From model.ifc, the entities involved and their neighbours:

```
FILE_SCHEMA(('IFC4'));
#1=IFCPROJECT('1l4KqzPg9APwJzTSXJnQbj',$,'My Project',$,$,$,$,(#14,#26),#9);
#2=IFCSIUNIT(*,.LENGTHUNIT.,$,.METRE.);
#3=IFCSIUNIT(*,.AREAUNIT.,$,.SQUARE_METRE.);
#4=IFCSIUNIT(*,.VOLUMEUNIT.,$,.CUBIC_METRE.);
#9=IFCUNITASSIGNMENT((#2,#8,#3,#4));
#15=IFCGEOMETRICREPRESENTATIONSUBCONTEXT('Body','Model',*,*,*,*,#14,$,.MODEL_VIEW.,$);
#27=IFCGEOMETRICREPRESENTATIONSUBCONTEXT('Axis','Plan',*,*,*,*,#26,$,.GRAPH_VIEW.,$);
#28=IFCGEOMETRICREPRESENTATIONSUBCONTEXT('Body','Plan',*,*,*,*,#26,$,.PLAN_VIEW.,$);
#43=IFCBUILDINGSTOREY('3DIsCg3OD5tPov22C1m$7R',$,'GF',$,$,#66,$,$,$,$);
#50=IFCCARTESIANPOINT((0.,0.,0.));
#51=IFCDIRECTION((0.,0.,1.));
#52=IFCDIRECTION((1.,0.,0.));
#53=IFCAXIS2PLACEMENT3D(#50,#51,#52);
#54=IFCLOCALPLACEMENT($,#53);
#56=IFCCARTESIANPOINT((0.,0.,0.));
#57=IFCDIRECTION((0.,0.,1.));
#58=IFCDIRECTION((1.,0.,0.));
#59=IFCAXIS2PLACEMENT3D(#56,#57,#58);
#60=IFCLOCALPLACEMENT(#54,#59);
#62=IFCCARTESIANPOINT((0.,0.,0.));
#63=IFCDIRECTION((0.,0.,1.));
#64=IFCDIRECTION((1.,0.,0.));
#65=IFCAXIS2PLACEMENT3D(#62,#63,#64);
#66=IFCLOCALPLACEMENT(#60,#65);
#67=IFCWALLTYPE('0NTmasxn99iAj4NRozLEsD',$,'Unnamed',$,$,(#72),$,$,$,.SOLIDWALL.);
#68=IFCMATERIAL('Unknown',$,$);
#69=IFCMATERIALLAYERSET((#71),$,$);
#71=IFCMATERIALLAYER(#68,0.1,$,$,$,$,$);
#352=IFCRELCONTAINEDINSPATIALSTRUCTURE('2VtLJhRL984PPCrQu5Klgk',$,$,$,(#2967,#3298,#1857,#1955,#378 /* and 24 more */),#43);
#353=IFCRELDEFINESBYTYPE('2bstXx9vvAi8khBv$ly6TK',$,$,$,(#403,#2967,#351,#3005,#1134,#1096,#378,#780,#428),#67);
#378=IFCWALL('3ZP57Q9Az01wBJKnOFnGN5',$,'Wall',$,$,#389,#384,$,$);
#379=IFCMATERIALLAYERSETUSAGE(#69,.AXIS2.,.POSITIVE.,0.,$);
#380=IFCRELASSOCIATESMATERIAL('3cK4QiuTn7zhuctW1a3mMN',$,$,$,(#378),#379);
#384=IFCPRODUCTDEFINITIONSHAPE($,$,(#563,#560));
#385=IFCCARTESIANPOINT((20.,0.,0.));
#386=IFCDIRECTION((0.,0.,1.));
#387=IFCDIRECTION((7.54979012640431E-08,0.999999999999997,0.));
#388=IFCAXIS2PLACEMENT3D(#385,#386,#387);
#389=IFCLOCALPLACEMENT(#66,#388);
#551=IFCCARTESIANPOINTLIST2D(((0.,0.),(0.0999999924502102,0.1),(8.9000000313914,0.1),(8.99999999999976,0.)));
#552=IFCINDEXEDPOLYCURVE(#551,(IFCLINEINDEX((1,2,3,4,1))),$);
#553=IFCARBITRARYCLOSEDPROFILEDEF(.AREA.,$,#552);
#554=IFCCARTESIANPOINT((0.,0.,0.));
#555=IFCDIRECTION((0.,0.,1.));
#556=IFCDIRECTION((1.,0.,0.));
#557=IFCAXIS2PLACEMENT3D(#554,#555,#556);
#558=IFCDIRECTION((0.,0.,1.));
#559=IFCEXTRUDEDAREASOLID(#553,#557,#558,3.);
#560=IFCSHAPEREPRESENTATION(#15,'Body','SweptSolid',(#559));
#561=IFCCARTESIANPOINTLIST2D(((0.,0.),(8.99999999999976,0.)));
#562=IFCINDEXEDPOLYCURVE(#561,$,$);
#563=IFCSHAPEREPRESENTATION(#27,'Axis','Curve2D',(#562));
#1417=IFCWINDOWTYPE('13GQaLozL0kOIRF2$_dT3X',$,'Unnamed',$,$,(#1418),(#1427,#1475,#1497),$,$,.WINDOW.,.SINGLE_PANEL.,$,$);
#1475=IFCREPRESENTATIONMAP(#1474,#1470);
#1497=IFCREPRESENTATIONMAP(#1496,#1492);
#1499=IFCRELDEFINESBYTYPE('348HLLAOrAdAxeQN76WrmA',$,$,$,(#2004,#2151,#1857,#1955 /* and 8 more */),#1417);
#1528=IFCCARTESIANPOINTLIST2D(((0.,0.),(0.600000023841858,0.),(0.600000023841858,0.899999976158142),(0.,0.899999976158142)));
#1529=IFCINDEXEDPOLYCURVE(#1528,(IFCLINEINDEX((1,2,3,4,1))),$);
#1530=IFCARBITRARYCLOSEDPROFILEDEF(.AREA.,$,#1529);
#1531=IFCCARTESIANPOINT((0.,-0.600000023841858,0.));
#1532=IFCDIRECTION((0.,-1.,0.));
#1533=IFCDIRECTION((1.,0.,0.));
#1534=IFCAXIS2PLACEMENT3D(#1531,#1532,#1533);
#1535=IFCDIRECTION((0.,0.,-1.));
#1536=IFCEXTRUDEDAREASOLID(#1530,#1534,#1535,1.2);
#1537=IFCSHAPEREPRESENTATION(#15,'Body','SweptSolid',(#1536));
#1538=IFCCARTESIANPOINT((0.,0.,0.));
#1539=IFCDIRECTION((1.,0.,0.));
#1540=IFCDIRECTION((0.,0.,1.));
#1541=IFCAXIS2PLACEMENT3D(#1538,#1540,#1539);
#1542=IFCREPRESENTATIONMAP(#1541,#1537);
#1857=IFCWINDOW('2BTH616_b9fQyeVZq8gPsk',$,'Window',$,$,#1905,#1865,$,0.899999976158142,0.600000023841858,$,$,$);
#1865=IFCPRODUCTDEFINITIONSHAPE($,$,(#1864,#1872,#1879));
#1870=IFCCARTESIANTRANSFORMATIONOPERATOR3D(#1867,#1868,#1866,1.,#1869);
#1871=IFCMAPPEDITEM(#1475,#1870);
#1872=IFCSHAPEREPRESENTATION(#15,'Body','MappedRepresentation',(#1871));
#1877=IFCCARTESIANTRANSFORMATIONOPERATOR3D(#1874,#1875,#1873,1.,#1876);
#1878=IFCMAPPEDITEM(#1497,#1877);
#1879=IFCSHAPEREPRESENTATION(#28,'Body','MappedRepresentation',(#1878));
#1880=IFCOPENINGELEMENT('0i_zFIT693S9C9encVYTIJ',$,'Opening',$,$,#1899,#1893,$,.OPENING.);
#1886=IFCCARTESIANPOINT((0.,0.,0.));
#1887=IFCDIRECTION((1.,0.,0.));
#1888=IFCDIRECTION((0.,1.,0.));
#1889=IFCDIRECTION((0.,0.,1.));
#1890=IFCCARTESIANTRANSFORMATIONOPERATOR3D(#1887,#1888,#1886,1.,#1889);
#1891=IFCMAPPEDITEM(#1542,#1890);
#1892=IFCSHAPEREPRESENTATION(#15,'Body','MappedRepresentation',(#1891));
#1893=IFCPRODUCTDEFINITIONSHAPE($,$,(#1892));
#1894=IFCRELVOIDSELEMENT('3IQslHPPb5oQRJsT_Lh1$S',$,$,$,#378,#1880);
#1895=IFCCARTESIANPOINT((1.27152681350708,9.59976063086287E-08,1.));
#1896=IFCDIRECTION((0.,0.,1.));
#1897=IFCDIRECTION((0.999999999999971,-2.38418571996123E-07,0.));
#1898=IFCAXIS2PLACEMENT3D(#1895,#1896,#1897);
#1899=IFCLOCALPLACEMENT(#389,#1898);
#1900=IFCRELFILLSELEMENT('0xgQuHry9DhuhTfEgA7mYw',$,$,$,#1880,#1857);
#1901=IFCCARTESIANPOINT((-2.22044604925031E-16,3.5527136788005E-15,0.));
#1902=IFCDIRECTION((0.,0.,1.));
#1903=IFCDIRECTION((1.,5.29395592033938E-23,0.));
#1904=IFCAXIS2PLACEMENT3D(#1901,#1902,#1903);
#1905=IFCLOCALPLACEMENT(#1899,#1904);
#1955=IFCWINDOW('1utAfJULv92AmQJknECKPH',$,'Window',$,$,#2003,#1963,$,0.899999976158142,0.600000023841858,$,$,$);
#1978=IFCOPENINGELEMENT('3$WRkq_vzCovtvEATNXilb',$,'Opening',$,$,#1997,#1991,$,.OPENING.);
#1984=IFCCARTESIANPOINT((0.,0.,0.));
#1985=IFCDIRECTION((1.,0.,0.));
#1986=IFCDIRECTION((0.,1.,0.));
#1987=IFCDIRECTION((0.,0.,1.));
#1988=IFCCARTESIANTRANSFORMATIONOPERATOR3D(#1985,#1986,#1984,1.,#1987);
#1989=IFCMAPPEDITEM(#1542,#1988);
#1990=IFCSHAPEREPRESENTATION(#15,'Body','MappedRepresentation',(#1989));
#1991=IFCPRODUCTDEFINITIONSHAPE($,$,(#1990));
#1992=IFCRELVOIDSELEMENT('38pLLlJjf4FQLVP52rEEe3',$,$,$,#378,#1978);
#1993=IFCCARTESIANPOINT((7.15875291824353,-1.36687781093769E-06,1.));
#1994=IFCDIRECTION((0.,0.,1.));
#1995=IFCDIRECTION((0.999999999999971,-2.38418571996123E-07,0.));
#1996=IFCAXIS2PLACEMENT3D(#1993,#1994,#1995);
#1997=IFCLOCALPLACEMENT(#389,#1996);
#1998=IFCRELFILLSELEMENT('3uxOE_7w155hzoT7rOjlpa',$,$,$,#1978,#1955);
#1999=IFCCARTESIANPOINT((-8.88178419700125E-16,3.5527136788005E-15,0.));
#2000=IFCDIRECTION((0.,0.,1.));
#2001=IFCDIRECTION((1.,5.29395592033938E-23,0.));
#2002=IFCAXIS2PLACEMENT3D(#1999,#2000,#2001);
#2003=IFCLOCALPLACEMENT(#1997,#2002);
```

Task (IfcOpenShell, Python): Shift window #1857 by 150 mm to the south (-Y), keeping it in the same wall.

```python
import ifcopenshell
import ifcopenshell.api.geometry
import ifcopenshell.util.placement
import ifcopenshell.util.unit

model = ifcopenshell.open("model.ifc")
unit_scale = ifcopenshell.util.unit.calculate_unit_scale(model)

window = model.by_guid("2BTH616_b9fQyeVZq8gPsk")
opening = window.FillsVoids[0].RelatingOpeningElement
wall = opening.VoidsElements[0].RelatingBuildingElement

wall_matrix = ifcopenshell.util.placement.get_local_placement(wall.ObjectPlacement)
shift = wall_matrix[:3, 0] * -0.15 / unit_scale
before = ifcopenshell.util.placement.get_local_placement(window.ObjectPlacement)[:3, 3].copy()

# The window is placed relative to its opening, so it follows when the opening moves.
matrix = ifcopenshell.util.placement.get_local_placement(opening.ObjectPlacement)
matrix[:3, 3] += shift
ifcopenshell.api.geometry.edit_object_placement(
    model, product=opening, matrix=matrix, is_si=False, should_transform_children=True
)

after = ifcopenshell.util.placement.get_local_placement(window.ObjectPlacement)[:3, 3]
print("window moved by", (after - before).round(3) + 0.0)

model.write("model_v2.ifc")
```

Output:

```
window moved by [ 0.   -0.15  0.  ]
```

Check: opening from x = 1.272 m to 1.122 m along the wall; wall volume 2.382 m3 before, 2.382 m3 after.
